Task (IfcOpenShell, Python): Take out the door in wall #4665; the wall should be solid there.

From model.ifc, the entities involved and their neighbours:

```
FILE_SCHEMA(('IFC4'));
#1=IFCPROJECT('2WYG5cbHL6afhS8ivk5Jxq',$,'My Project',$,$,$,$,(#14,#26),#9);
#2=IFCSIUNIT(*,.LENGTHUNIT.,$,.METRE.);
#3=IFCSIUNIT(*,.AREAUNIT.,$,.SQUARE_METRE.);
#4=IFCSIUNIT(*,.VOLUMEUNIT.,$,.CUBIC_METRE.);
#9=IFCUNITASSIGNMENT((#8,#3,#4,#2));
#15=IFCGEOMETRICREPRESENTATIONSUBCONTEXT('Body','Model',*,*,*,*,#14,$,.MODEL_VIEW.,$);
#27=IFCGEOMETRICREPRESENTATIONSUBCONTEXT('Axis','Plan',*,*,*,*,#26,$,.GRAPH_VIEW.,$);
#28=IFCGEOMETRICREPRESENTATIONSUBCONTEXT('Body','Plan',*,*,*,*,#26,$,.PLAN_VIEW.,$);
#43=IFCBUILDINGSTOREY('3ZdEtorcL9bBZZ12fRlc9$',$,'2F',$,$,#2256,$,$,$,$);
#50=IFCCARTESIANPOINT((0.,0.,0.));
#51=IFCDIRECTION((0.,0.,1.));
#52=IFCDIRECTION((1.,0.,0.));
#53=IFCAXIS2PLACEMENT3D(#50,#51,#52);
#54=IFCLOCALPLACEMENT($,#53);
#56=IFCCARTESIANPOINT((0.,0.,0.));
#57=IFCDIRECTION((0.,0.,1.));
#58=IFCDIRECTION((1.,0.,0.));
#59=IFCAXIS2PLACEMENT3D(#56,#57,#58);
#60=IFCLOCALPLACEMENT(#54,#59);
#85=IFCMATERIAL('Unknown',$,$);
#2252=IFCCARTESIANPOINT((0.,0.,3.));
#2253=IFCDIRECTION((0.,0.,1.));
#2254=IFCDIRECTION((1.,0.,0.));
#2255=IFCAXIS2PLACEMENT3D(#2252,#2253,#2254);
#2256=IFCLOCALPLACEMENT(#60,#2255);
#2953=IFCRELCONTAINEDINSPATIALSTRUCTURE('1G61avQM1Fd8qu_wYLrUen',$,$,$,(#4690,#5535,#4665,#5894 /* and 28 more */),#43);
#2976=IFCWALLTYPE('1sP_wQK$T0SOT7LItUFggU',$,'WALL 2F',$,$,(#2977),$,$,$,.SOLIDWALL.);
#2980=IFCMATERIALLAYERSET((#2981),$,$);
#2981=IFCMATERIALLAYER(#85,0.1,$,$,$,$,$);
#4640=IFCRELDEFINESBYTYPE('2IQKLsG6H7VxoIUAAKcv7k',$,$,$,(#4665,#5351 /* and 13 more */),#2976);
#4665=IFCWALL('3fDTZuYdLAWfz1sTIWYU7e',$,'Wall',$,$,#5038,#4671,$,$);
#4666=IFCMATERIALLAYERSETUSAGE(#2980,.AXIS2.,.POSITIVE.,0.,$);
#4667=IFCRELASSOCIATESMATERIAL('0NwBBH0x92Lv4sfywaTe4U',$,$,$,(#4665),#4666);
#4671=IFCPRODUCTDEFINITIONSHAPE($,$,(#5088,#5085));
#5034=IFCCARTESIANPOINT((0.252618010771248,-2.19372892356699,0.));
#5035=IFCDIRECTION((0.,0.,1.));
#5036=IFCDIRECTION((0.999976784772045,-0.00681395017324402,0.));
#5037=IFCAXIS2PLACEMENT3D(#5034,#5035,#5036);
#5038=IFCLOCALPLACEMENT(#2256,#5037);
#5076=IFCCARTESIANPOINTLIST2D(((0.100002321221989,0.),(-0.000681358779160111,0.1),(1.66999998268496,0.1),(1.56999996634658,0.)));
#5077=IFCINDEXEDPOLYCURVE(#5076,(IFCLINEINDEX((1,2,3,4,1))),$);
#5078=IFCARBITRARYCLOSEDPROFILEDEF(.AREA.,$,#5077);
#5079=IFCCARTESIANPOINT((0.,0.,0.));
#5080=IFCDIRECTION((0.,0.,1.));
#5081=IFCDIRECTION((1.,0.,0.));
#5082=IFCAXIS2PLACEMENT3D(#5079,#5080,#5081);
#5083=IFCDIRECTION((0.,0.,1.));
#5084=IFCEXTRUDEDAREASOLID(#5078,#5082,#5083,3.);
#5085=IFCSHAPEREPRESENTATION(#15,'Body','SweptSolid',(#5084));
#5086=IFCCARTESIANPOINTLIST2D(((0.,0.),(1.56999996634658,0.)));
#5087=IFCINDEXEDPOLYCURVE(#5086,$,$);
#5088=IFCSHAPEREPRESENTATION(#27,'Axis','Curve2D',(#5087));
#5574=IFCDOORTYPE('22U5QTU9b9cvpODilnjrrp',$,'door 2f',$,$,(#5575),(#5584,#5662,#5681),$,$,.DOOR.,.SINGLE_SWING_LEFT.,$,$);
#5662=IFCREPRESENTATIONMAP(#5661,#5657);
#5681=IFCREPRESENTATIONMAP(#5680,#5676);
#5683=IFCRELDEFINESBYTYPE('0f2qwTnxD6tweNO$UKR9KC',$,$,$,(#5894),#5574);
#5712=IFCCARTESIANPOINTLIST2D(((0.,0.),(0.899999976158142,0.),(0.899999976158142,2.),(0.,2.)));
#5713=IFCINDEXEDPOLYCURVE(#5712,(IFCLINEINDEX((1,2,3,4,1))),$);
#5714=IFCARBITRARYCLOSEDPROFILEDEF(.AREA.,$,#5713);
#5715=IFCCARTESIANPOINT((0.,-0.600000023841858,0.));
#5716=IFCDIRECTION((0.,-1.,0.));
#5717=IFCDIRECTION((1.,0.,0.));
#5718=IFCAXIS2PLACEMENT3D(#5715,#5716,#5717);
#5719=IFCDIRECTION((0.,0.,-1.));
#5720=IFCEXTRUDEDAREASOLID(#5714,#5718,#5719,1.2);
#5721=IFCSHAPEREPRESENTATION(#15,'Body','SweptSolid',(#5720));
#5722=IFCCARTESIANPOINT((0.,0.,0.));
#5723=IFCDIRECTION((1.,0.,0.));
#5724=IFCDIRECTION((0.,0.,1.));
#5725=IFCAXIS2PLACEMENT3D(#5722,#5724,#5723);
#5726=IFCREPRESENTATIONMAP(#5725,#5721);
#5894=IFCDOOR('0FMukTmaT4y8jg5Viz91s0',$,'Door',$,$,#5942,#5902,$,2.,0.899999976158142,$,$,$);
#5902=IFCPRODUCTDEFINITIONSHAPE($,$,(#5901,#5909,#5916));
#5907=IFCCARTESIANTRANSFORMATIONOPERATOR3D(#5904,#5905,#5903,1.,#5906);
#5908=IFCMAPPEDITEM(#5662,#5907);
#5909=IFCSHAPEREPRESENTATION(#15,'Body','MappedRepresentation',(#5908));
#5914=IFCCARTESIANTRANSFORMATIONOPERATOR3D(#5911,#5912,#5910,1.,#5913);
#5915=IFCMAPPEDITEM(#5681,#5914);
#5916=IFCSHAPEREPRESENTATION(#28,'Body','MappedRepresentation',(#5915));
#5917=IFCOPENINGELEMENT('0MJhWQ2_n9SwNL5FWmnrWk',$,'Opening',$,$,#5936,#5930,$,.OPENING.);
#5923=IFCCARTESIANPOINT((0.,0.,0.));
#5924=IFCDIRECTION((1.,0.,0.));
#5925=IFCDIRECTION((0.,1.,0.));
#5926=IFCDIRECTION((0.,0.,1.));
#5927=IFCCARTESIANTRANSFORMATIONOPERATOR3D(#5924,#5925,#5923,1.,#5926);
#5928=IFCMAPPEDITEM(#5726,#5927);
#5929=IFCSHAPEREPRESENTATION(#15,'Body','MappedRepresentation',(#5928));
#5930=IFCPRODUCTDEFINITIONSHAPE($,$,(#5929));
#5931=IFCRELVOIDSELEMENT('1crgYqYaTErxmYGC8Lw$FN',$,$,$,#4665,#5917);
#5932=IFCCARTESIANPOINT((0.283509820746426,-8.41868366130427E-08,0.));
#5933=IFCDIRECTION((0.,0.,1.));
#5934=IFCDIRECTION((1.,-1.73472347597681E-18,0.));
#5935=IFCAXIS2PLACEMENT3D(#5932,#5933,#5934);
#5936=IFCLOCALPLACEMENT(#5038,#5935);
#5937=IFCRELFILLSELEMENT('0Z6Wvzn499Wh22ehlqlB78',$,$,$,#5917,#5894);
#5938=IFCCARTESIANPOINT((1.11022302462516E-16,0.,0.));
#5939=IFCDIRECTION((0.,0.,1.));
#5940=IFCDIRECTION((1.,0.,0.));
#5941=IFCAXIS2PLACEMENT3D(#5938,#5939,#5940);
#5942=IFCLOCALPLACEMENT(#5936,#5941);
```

```python
import ifcopenshell
import ifcopenshell.api.feature
import ifcopenshell.api.root
import ifcopenshell.geom
import ifcopenshell.util.shape

model = ifcopenshell.open("model.ifc")
settings = ifcopenshell.geom.settings()


def volume(element):
    """Net volume in cubic metres, openings subtracted."""
    shape = ifcopenshell.geom.create_shape(settings, element)
    return ifcopenshell.util.shape.get_volume(shape.geometry)


door = model.by_guid("0FMukTmaT4y8jg5Viz91s0")
opening = door.FillsVoids[0].RelatingOpeningElement
wall = opening.VoidsElements[0].RelatingBuildingElement
before = volume(wall)

ifcopenshell.api.root.remove_product(model, product=door)
ifcopenshell.api.feature.remove_feature(model, feature=opening)

after = volume(wall)

print(f"wall volume {before:.3f} -> {after:.3f} m3")

model.write("model_updated.ifc")
```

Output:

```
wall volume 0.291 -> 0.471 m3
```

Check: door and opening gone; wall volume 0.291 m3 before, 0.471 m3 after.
